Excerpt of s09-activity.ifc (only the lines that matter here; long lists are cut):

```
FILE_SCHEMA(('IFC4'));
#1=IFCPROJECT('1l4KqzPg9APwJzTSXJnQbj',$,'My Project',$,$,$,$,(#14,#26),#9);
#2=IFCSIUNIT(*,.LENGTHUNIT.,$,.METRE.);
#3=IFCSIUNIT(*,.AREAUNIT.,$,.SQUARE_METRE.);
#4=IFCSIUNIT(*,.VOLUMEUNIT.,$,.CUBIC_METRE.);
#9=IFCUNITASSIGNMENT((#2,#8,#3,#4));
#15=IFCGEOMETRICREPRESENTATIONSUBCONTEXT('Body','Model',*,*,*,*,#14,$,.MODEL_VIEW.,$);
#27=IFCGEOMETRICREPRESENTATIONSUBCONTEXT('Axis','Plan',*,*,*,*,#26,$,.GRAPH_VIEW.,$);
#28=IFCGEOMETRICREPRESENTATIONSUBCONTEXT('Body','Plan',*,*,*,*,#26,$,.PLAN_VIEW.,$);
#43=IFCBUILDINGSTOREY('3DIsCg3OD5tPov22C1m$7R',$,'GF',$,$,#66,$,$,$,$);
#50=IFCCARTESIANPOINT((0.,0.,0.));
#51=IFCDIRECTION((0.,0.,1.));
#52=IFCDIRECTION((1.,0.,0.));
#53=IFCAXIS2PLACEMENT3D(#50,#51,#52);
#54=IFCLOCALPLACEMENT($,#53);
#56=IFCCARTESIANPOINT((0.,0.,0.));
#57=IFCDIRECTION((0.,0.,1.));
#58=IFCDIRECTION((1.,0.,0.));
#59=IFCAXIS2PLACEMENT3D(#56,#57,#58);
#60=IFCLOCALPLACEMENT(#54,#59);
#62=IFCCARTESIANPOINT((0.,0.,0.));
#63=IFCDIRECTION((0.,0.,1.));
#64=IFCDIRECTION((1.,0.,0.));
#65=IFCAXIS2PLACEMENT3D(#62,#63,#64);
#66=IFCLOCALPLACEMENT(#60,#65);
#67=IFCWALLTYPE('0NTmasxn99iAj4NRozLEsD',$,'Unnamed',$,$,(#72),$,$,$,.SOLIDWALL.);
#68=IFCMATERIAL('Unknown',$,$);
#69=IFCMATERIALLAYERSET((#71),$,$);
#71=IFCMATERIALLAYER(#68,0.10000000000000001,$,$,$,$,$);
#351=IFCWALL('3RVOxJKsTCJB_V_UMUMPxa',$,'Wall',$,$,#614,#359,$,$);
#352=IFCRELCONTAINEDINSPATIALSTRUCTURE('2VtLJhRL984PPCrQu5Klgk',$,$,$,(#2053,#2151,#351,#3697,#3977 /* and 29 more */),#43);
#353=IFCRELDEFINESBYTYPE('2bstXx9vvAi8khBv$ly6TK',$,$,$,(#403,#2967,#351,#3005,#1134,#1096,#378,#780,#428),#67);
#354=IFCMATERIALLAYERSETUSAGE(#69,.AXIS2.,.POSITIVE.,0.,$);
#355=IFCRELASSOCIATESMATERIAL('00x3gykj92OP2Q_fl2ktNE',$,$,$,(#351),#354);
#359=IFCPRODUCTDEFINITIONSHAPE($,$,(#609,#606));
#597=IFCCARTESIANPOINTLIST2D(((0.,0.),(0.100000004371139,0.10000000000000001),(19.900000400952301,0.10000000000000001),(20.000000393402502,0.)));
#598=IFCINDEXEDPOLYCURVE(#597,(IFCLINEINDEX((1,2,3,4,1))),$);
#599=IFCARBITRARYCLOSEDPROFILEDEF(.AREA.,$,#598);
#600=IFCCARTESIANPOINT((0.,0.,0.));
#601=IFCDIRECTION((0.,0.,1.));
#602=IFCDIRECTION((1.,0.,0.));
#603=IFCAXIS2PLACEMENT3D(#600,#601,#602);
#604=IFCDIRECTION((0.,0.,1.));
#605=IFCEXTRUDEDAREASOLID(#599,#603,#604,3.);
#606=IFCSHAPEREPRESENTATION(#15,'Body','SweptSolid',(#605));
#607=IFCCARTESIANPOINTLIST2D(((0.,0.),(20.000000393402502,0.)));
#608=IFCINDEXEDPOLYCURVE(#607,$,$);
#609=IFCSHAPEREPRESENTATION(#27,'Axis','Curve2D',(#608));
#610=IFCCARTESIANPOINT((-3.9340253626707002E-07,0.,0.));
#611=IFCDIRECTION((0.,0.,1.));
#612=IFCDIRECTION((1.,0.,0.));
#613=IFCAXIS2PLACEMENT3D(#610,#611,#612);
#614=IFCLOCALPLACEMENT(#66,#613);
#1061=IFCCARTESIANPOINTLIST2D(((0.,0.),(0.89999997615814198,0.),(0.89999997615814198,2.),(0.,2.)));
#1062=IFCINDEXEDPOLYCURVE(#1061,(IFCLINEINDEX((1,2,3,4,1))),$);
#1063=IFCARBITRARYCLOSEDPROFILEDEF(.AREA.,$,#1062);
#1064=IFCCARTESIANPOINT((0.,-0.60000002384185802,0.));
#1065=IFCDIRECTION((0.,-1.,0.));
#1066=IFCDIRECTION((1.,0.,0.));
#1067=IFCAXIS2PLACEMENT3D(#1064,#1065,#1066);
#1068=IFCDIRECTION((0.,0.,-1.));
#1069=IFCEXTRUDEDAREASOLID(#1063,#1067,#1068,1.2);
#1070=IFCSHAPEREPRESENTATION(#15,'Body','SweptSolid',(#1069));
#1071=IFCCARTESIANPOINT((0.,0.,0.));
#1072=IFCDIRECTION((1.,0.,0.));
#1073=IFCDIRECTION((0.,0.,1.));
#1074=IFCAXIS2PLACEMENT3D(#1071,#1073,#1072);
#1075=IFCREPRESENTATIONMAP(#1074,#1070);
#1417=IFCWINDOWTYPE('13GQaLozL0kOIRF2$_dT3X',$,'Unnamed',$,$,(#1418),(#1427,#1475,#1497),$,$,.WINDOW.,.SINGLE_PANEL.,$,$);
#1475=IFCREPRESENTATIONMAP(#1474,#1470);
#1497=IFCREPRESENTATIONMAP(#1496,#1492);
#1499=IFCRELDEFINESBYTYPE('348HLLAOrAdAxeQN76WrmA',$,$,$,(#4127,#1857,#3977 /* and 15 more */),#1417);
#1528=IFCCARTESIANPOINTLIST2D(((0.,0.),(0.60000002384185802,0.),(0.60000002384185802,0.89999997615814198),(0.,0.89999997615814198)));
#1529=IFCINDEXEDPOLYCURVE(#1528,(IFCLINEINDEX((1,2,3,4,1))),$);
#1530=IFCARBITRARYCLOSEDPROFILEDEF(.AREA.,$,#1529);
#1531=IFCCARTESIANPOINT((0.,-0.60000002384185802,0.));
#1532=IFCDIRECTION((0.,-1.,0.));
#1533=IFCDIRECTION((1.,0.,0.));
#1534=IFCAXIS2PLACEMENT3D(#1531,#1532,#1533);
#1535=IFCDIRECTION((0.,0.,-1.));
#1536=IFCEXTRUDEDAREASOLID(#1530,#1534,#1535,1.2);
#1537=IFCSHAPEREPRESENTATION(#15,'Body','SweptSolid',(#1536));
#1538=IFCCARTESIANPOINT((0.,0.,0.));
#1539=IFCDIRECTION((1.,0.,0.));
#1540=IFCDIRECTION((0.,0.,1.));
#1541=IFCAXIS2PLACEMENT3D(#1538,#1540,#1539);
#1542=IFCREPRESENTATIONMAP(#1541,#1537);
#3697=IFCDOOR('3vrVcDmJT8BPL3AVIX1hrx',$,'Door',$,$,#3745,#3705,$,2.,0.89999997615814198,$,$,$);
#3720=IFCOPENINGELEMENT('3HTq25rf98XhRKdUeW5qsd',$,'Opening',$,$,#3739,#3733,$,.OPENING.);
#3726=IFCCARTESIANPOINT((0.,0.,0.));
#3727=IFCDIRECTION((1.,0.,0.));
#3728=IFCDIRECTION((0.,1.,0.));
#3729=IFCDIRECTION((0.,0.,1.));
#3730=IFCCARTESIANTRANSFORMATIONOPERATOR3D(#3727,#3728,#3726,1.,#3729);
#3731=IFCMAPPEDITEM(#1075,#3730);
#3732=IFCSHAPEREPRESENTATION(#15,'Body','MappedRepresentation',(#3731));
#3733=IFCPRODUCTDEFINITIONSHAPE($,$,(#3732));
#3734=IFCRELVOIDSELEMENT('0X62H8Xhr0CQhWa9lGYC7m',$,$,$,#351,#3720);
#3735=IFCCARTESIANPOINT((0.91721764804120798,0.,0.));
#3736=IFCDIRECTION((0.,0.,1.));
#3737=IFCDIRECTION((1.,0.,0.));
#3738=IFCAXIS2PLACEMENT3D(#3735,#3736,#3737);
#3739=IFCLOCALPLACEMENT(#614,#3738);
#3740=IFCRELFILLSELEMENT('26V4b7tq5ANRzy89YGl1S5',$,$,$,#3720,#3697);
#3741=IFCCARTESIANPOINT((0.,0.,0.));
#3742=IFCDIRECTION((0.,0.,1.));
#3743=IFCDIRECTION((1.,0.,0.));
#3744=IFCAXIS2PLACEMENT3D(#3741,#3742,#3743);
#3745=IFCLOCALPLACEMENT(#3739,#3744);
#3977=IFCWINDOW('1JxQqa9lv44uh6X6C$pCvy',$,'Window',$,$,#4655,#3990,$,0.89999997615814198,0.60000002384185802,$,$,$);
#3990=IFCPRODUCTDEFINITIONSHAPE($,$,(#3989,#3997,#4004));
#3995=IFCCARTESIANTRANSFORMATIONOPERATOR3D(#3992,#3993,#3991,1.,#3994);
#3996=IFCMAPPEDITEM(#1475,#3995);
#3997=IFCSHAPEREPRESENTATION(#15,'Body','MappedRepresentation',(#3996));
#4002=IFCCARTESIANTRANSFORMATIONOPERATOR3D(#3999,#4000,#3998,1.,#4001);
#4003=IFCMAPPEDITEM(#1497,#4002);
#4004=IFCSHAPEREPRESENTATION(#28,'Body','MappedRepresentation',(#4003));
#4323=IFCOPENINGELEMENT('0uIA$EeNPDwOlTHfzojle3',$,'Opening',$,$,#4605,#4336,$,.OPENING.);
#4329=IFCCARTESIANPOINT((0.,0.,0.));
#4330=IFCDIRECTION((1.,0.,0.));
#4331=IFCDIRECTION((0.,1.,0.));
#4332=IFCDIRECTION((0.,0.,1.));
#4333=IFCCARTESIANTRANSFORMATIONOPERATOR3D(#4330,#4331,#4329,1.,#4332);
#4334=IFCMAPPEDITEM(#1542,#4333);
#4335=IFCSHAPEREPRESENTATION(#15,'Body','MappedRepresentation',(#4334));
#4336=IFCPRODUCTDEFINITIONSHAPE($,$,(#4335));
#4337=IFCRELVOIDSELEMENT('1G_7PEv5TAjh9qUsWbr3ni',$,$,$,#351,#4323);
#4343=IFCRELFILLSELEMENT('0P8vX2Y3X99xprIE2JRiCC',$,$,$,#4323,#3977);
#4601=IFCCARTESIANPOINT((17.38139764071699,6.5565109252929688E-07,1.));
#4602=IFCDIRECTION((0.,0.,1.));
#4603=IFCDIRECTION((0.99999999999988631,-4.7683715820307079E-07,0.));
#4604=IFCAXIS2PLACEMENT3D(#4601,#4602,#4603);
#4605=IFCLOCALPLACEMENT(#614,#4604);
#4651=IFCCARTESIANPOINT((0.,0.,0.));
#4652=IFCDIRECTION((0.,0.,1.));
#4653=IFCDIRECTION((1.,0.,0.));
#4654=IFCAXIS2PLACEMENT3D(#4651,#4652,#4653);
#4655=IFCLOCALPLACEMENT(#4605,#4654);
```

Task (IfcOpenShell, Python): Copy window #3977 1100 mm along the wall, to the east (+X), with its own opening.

```python
import ifcopenshell
import ifcopenshell.api.feature
import ifcopenshell.api.geometry
import ifcopenshell.api.root
import ifcopenshell.geom
import ifcopenshell.util.element
import ifcopenshell.util.placement
import ifcopenshell.util.shape

model = ifcopenshell.open("s09-activity.ifc")
settings = ifcopenshell.geom.settings()


def volume(element):
    """Net volume in cubic metres, openings subtracted."""
    shape = ifcopenshell.geom.create_shape(settings, element)
    return ifcopenshell.util.shape.get_volume(shape.geometry)


window = model.by_id(3977)
opening = window.FillsVoids[0].RelatingOpeningElement
wall = opening.VoidsElements[0].RelatingBuildingElement
before = volume(wall)
shift = ifcopenshell.util.placement.get_local_placement(wall.ObjectPlacement)[:3, 0] * 1.1

# copy_class copies the void relationship, type, container and properties, but no geometry.
new_opening = ifcopenshell.api.root.copy_class(model, product=opening)
new_opening.Representation = ifcopenshell.util.element.copy_deep(
    model, opening.Representation, exclude=["IfcGeometricRepresentationContext", "IfcRepresentationMap"]
)
new_window = ifcopenshell.api.root.copy_class(model, product=window)
new_window.Representation = ifcopenshell.util.element.copy_deep(
    model, window.Representation, exclude=["IfcGeometricRepresentationContext", "IfcRepresentationMap"]
)
ifcopenshell.api.feature.add_filling(model, opening=new_opening, element=new_window)

for old, new in ((opening, new_opening), (window, new_window)):
    matrix = ifcopenshell.util.placement.get_local_placement(old.ObjectPlacement)
    matrix[:3, 3] += shift
    ifcopenshell.api.geometry.edit_object_placement(model, product=new, matrix=matrix, is_si=False)

after = volume(wall)

print(f"wall volume {before:.3f} -> {after:.3f} m3")

model.write("s09-activity_v2.ifc")
```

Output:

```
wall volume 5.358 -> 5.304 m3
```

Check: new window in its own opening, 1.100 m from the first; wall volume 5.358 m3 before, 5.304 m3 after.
